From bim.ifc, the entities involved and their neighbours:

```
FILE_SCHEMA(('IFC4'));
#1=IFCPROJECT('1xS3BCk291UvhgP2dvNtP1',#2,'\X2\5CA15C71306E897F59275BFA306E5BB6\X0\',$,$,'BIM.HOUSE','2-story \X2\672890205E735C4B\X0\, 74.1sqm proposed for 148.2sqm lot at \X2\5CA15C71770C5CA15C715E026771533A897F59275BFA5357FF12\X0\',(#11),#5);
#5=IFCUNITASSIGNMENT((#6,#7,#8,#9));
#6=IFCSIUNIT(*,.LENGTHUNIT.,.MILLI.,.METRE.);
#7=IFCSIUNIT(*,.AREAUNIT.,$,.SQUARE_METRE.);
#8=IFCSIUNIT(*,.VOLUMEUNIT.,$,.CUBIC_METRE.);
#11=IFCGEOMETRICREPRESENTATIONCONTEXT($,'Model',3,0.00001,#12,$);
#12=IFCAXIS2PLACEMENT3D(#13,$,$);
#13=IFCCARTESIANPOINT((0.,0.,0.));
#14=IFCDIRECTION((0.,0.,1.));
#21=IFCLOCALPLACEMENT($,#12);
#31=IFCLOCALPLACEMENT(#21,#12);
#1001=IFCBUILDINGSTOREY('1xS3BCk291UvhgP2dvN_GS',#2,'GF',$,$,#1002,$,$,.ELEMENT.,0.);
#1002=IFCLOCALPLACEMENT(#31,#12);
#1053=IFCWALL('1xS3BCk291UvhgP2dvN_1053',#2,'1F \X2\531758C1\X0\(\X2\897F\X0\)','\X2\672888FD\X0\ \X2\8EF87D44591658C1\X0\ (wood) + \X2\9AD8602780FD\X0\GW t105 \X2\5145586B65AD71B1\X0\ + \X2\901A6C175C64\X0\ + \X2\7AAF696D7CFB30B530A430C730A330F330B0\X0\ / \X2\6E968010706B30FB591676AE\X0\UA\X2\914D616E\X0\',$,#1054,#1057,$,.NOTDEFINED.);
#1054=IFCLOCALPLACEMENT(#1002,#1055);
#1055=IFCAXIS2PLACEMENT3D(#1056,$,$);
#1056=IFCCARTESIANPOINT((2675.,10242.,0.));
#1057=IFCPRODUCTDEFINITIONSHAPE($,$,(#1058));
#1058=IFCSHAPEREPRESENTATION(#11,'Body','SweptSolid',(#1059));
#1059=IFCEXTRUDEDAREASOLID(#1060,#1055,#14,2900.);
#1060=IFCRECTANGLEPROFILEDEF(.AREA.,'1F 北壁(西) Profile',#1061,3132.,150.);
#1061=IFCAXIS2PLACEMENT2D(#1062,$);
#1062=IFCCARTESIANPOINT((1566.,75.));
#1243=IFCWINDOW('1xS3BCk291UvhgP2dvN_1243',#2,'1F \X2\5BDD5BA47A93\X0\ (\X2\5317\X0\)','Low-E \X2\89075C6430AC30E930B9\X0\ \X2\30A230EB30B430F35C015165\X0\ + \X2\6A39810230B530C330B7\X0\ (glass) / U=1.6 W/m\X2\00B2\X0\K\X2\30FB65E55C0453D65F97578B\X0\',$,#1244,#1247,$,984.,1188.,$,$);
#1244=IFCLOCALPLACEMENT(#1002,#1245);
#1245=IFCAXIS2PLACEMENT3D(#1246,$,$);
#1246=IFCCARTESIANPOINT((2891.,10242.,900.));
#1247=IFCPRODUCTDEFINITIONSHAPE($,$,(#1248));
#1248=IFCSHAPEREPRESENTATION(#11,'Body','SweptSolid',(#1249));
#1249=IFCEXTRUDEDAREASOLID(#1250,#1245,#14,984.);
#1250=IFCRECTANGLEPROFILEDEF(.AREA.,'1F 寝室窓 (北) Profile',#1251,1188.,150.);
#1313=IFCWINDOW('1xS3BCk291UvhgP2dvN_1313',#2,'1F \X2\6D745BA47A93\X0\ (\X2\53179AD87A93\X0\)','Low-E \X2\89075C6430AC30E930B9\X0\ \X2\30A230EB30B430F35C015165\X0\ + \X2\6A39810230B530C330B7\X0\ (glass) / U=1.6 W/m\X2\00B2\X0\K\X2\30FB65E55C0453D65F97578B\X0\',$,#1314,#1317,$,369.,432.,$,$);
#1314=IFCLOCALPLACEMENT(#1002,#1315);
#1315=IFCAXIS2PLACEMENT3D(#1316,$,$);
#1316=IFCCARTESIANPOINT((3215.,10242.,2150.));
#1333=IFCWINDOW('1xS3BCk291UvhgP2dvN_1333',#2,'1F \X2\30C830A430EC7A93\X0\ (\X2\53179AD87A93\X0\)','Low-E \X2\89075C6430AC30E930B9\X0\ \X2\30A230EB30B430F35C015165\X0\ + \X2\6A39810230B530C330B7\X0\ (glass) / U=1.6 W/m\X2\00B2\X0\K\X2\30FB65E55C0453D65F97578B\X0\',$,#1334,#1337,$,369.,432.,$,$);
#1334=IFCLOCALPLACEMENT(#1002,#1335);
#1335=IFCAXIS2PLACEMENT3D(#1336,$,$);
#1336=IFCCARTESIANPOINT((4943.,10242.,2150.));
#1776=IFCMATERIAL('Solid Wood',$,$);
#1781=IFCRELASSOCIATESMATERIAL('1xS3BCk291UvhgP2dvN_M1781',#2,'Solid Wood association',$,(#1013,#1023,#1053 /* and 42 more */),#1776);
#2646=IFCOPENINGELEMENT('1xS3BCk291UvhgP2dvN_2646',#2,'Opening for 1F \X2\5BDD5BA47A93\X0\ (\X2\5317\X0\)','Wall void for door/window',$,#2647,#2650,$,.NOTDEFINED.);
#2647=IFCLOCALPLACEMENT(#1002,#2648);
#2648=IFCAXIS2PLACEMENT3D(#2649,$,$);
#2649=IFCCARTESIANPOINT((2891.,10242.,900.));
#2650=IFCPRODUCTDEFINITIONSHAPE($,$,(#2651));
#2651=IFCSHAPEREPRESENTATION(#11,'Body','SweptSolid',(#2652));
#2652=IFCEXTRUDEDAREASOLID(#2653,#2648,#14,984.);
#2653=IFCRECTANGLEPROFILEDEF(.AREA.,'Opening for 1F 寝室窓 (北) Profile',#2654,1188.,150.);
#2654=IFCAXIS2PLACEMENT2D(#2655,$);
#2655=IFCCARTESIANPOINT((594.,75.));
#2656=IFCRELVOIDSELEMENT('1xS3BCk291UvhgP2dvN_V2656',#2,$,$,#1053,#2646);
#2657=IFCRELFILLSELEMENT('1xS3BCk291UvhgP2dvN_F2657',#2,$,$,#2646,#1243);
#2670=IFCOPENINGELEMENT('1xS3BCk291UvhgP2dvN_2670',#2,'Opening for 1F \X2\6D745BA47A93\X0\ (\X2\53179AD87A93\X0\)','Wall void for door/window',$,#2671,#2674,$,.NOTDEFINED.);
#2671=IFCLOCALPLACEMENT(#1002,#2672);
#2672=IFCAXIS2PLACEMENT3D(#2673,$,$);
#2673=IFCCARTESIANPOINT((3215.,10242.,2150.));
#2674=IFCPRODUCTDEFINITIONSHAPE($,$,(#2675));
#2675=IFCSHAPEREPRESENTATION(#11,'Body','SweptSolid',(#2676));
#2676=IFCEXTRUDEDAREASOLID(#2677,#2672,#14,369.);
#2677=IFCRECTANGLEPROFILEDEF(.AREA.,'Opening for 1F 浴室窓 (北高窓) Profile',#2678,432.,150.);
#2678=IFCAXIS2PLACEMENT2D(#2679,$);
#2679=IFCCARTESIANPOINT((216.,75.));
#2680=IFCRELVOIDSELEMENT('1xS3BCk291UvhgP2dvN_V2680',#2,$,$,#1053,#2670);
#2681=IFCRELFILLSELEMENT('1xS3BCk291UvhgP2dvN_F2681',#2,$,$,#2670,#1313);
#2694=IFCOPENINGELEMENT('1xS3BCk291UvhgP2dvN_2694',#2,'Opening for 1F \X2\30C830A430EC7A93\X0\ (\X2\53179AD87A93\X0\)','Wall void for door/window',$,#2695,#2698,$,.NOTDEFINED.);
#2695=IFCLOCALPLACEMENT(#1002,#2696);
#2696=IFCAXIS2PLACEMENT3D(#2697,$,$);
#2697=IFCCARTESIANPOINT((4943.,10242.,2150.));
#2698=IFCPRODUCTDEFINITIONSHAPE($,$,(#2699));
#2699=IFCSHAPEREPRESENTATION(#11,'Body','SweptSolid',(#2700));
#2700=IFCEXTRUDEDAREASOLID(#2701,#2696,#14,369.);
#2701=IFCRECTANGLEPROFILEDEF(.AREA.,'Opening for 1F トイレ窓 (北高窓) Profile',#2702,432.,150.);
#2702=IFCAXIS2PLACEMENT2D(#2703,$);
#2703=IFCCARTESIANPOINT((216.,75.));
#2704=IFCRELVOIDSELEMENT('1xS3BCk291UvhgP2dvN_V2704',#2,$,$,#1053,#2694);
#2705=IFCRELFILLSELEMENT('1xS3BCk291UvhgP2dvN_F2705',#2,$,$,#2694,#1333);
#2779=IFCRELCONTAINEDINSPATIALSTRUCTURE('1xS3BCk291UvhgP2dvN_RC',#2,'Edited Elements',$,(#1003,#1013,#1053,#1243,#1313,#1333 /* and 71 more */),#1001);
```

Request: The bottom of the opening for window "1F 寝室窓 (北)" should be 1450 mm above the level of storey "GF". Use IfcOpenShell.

```python
import numpy as np
import ifcopenshell
import ifcopenshell.api.geometry
import ifcopenshell.geom
import ifcopenshell.util.element
import ifcopenshell.util.placement
import ifcopenshell.util.shape
import ifcopenshell.util.unit

model = ifcopenshell.open("bim.ifc")
unit_scale = ifcopenshell.util.unit.calculate_unit_scale(model)

window = model.by_guid("1xS3BCk291UvhgP2dvN_1243")
opening = window.FillsVoids[0].RelatingOpeningElement
storey = ifcopenshell.util.element.get_container(window, ifc_class="IfcBuildingStorey")
level = ifcopenshell.util.placement.get_local_placement(storey.ObjectPlacement)[2, 3]

# The opening's origin need not be at the sill, so measure its lowest point.
shape = ifcopenshell.geom.create_shape(ifcopenshell.geom.settings(), opening)
bottom = ifcopenshell.util.shape.get_shape_bottom_elevation(shape, shape.geometry) / unit_scale
dz = level + 1.45 / unit_scale - bottom

shift = np.array([0.0, 0.0, dz])
# The window is not placed relative to its opening, so move both.
for product in (opening, window):
    matrix = ifcopenshell.util.placement.get_local_placement(product.ObjectPlacement)
    matrix[:3, 3] += shift
    ifcopenshell.api.geometry.edit_object_placement(model, product=product, matrix=matrix, is_si=False)

print(f"moved by {dz * unit_scale:+.3f} m")

model.write("bim-out.ifc")
```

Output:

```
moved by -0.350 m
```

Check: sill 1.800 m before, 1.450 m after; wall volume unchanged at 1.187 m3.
